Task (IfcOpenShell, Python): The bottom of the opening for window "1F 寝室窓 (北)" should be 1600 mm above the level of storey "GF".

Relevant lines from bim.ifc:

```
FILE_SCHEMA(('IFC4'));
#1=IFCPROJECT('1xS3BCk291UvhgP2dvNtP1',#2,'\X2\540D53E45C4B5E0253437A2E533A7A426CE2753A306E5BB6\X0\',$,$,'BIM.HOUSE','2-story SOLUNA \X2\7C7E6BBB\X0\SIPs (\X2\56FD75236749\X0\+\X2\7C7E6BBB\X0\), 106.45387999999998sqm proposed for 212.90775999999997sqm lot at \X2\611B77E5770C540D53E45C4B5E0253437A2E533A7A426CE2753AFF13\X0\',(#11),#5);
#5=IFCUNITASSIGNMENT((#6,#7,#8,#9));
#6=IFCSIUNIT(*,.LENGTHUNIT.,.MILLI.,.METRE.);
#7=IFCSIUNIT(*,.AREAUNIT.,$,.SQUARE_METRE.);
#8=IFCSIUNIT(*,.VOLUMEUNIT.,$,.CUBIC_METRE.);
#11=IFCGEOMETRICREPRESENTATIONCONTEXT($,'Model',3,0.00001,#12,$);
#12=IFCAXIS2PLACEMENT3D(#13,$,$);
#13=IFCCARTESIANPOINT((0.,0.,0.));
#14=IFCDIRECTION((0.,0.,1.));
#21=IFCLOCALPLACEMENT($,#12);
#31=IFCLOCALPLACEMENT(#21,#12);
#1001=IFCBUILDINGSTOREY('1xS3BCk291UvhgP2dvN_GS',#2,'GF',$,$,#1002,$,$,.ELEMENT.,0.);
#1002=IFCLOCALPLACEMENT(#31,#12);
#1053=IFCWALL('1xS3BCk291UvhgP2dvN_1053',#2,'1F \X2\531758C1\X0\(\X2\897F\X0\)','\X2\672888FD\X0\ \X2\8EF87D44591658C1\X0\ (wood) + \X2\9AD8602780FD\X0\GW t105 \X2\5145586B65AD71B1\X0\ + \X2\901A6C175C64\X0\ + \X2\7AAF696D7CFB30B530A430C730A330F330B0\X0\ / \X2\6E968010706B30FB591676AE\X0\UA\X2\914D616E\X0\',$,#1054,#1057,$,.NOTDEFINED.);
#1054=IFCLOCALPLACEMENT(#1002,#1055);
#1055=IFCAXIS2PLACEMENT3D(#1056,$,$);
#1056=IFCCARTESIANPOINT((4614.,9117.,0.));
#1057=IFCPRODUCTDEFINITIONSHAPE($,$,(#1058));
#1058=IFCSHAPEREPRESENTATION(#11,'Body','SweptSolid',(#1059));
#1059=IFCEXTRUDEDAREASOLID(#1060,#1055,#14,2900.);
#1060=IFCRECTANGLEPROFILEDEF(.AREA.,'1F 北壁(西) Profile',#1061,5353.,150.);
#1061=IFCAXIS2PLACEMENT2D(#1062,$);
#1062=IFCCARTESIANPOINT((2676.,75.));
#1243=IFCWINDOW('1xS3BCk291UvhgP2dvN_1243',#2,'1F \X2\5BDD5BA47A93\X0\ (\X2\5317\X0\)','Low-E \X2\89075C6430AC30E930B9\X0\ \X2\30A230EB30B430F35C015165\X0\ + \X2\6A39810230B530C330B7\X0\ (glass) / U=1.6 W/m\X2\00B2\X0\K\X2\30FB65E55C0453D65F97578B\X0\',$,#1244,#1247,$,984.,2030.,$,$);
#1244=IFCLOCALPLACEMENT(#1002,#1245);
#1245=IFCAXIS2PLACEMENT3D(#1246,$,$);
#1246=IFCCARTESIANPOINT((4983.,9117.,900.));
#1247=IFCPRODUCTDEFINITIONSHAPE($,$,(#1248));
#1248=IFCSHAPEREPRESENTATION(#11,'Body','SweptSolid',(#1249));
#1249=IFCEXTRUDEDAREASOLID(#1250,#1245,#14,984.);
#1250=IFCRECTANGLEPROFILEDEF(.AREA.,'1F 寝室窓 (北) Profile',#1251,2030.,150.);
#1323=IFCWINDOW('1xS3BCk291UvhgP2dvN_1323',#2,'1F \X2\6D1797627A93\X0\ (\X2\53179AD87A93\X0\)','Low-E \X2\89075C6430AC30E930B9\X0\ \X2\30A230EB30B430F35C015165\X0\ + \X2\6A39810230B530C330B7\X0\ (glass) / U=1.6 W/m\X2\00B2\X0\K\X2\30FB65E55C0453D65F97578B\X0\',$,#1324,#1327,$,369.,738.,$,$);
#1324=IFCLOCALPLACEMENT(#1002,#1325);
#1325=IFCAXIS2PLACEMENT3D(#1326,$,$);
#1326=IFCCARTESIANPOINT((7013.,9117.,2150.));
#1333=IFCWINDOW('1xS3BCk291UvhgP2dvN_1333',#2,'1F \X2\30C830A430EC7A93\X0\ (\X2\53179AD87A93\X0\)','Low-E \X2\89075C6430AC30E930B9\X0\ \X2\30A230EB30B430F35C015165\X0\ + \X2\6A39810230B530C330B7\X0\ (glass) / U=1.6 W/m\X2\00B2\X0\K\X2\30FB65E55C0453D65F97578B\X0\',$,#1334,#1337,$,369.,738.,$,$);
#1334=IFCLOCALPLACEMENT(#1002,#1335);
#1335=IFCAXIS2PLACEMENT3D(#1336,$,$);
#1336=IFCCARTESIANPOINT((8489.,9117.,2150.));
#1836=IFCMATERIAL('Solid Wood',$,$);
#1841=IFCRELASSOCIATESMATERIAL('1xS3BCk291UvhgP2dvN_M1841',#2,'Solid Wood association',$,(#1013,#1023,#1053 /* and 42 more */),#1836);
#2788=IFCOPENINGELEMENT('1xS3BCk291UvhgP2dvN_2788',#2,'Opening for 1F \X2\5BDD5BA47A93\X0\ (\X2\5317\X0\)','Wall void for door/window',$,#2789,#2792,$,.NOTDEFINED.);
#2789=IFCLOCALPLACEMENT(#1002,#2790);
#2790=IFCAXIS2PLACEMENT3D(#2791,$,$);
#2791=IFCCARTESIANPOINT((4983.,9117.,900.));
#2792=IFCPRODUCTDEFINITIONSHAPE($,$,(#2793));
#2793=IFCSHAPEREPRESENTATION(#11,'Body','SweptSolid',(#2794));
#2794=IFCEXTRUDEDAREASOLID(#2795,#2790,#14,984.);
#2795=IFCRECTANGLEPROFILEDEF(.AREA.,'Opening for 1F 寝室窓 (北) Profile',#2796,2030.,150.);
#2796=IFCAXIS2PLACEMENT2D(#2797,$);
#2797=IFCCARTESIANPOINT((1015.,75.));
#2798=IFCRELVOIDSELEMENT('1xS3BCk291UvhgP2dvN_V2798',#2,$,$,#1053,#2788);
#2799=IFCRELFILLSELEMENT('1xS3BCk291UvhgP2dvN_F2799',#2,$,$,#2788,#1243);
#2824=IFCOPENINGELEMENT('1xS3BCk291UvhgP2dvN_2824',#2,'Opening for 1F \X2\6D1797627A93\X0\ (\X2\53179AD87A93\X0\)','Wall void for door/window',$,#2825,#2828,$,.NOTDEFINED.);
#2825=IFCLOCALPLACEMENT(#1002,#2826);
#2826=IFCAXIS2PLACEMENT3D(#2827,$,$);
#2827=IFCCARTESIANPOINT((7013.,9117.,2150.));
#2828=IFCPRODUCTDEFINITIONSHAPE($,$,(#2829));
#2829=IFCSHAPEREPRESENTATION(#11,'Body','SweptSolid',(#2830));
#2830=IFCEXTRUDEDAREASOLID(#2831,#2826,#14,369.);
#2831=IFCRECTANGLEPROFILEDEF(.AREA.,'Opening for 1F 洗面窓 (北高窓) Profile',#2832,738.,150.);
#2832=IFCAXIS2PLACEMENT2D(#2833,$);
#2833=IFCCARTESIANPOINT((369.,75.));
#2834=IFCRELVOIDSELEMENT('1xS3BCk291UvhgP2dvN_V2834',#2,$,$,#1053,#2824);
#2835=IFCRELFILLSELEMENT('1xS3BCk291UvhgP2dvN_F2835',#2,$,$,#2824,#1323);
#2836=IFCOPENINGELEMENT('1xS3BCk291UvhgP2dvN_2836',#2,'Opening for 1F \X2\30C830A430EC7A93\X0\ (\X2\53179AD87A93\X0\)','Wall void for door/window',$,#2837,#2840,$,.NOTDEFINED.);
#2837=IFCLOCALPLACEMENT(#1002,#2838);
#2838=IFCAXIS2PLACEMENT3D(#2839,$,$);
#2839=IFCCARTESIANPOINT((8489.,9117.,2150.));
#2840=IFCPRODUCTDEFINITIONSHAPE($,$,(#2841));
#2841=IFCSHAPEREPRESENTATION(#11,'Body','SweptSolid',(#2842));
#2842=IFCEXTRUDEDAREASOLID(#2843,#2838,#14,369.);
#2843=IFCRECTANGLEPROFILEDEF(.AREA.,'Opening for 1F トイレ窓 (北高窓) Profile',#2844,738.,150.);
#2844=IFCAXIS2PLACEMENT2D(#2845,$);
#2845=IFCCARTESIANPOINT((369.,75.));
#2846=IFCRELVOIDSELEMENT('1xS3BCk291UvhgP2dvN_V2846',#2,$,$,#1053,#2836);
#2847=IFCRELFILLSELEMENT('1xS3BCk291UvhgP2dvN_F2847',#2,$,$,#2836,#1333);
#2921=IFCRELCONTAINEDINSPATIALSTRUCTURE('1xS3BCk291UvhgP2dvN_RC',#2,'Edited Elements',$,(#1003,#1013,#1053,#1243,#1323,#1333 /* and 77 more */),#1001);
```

```python
import numpy as np
import ifcopenshell
import ifcopenshell.api.geometry
import ifcopenshell.geom
import ifcopenshell.util.element
import ifcopenshell.util.placement
import ifcopenshell.util.shape
import ifcopenshell.util.unit

model = ifcopenshell.open("bim.ifc")
unit_scale = ifcopenshell.util.unit.calculate_unit_scale(model)

window = model.by_guid("1xS3BCk291UvhgP2dvN_1243")
opening = window.FillsVoids[0].RelatingOpeningElement
storey = ifcopenshell.util.element.get_container(window, ifc_class="IfcBuildingStorey")
level = ifcopenshell.util.placement.get_local_placement(storey.ObjectPlacement)[2, 3]

# The opening's origin need not be at the sill, so measure its lowest point.
shape = ifcopenshell.geom.create_shape(ifcopenshell.geom.settings(), opening)
bottom = ifcopenshell.util.shape.get_shape_bottom_elevation(shape, shape.geometry) / unit_scale
dz = level + 1600.0 - bottom

shift = np.array([0.0, 0.0, dz])
# The window is not placed relative to its opening, so move both.
for product in (opening, window):
    matrix = ifcopenshell.util.placement.get_local_placement(product.ObjectPlacement)
    matrix[:3, 3] += shift
    ifcopenshell.api.geometry.edit_object_placement(model, product=product, matrix=matrix, is_si=False)

print(f"moved by {dz * unit_scale:+.3f} m")

model.write("bim_updated.ifc")
```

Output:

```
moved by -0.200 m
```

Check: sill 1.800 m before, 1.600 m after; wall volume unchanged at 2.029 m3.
